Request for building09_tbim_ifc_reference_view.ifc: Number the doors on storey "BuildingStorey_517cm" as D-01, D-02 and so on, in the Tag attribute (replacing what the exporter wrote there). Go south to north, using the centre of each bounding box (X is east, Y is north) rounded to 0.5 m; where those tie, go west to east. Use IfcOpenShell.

First a look at what the model holds.

```python
import ifcopenshell
import ifcopenshell.util.element
import ifcopenshell.util.placement

model = ifcopenshell.open("building09_tbim_ifc_reference_view.ifc")
print(model.schema)
storey = next(s for s in model.by_type("IfcBuildingStorey") if s.Name == "BuildingStorey_517cm")
doors = [e for e in ifcopenshell.util.element.get_decomposition(storey) if e.is_a("IfcDoor")]
for e in sorted(doors, key=lambda e: e.id()):
    origin = ifcopenshell.util.placement.get_local_placement(e.ObjectPlacement)[:3, 3]
    print(e.id(), e.Tag, e.Name, origin.round(2) + 0.0, sep=" | ")
```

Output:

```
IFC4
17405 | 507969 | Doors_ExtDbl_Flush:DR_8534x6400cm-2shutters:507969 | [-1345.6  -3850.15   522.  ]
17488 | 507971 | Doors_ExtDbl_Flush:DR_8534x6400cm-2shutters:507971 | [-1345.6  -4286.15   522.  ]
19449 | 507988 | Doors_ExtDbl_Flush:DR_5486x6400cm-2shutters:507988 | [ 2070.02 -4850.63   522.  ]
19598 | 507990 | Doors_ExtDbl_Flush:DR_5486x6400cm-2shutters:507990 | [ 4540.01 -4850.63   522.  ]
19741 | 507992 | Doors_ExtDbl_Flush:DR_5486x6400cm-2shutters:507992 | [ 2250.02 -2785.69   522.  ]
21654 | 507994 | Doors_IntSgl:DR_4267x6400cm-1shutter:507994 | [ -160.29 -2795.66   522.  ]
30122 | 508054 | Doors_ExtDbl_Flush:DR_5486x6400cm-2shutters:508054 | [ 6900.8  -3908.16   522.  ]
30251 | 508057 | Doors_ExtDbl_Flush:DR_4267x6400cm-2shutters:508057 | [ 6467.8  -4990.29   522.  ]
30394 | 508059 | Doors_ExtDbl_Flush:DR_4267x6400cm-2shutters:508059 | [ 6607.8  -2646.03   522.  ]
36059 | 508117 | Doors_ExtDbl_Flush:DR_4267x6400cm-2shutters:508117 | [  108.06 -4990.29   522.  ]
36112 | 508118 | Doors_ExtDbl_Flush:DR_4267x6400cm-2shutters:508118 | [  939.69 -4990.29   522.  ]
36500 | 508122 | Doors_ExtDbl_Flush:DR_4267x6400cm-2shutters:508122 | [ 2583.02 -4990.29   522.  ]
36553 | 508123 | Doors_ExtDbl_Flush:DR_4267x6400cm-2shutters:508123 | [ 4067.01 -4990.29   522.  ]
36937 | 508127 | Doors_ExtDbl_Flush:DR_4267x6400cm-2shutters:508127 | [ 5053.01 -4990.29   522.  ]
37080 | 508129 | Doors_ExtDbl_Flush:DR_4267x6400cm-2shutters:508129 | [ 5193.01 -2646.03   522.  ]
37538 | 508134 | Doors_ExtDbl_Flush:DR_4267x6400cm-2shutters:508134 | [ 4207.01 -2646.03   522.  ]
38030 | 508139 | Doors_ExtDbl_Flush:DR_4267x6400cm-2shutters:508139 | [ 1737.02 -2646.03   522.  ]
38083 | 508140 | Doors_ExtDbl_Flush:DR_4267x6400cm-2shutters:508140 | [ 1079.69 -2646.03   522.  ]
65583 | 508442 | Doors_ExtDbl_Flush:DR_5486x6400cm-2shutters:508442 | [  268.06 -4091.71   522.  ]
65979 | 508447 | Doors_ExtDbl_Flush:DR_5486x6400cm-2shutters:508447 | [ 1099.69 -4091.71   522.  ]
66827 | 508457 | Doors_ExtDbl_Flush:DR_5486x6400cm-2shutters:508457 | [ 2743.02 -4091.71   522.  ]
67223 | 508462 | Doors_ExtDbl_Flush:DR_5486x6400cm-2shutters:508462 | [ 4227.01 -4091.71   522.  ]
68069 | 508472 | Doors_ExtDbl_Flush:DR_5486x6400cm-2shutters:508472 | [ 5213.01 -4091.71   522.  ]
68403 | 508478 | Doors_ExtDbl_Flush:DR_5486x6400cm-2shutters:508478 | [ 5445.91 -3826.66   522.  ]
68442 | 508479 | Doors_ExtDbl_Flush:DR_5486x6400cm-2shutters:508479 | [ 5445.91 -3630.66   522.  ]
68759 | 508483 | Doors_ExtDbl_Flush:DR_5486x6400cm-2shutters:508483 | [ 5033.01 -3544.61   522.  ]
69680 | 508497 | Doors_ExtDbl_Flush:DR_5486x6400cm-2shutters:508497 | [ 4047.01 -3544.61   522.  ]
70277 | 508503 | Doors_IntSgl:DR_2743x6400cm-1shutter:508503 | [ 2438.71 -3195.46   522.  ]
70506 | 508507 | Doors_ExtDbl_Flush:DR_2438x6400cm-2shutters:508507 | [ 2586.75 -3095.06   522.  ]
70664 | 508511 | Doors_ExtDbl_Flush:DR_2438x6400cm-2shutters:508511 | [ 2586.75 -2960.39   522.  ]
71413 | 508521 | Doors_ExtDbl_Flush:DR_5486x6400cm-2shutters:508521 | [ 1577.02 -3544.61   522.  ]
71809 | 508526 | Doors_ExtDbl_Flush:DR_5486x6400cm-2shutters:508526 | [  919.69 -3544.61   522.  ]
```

```python
import ifcopenshell
import ifcopenshell.geom
import ifcopenshell.util.element
import ifcopenshell.util.shape

model = ifcopenshell.open("building09_tbim_ifc_reference_view.ifc")
settings = ifcopenshell.geom.settings()
settings.set("use-world-coords", True)


def centre(element):
    shape = ifcopenshell.geom.create_shape(settings, element)
    return ifcopenshell.util.shape.get_bbox_centroid(shape.geometry)


storey = next(s for s in model.by_type("IfcBuildingStorey") if s.Name == "BuildingStorey_517cm")
doors = [e for e in ifcopenshell.util.element.get_decomposition(storey) if e.is_a("IfcDoor")]

# Insertion points can sit at a corner or the storey origin, so sort by the geometry (in metres).
centres = {e: centre(e) for e in doors}
doors.sort(key=lambda e: (round(centres[e][1] / 0.5), centres[e][0]))

for i, e in enumerate(doors, start=1):
    number = f"D-{i:02d}"
    e.Tag = number
    print(e.id(), number)

model.write("building09_tbim_ifc_reference_view-out.ifc")
```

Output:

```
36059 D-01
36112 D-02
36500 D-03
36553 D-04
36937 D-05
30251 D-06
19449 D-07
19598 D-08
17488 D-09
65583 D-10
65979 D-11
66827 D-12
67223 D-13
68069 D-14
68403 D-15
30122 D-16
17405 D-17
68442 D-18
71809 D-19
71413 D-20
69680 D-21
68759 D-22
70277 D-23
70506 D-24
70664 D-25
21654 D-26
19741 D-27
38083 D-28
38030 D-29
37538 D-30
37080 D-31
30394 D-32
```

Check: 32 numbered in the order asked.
